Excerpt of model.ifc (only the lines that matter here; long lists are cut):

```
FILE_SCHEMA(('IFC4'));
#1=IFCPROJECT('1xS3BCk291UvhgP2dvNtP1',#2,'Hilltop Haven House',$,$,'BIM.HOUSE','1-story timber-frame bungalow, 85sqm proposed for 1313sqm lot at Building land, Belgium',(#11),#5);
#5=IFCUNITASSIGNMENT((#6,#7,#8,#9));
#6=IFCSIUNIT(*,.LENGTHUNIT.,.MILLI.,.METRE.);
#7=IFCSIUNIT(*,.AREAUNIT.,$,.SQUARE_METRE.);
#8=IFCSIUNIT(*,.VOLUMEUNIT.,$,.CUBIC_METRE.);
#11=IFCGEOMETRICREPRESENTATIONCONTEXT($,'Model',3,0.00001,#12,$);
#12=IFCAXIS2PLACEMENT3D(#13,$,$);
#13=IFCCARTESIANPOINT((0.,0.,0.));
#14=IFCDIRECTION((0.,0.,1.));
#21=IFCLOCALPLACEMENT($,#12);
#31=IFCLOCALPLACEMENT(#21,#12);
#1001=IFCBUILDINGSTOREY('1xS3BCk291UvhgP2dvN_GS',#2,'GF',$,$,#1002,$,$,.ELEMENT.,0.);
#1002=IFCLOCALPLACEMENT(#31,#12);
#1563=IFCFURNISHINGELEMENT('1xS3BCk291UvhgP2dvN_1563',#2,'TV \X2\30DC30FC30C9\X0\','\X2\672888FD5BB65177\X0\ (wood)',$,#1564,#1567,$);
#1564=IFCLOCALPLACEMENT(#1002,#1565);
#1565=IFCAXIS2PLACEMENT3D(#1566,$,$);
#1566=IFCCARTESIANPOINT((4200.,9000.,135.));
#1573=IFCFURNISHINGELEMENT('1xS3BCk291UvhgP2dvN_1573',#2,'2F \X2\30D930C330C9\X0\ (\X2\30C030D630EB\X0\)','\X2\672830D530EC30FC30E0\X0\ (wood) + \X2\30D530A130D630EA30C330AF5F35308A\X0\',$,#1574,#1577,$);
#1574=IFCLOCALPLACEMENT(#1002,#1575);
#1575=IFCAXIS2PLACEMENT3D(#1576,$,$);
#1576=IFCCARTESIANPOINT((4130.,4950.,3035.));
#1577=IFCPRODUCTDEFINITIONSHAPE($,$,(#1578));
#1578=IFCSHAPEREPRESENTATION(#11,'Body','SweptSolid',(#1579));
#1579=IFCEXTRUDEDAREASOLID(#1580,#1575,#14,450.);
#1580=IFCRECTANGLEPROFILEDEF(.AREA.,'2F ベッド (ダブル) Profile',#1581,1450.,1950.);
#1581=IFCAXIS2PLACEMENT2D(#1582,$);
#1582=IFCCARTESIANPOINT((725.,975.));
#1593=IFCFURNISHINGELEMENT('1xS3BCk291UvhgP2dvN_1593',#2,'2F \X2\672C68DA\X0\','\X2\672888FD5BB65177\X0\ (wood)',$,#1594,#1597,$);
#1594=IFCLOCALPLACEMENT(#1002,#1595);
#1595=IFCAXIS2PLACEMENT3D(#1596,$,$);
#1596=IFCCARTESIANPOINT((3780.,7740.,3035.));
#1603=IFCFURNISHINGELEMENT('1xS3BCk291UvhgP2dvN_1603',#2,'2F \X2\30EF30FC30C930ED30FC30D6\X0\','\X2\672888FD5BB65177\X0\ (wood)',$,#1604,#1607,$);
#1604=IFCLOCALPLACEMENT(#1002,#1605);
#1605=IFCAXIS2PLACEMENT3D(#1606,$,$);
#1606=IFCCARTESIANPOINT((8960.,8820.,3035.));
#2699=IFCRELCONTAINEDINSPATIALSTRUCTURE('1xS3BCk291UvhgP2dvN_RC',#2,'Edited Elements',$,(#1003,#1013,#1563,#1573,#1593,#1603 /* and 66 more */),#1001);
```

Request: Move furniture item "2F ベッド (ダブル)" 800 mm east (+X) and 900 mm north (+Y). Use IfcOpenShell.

```python
import ifcopenshell
import ifcopenshell.api.geometry
import ifcopenshell.util.placement
import ifcopenshell.util.unit

model = ifcopenshell.open("model.ifc")
unit_scale = ifcopenshell.util.unit.calculate_unit_scale(model)

item = model.by_guid("1xS3BCk291UvhgP2dvN_1573")
matrix = ifcopenshell.util.placement.get_local_placement(item.ObjectPlacement)
matrix[0, 3] += 0.8 / unit_scale
matrix[1, 3] += 0.9 / unit_scale
ifcopenshell.api.geometry.edit_object_placement(model, product=item, matrix=matrix, is_si=False)

print(ifcopenshell.util.placement.get_local_placement(item.ObjectPlacement).round(3) + 0.0)

model.write("model-out.ifc")
```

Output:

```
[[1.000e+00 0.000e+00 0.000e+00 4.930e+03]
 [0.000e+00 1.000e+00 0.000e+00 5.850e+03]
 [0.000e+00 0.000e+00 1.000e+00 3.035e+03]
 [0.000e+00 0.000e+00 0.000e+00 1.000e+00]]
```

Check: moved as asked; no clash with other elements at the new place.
